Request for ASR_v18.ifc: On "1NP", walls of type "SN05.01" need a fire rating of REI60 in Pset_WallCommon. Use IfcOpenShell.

First a look at what the model holds.

```python
import ifcopenshell
import ifcopenshell.util.element

model = ifcopenshell.open("ASR_v18.ifc")
print(model.schema)
storey = next(s for s in model.by_type("IfcBuildingStorey") if s.Name == "1NP")
walls = [e for e in ifcopenshell.util.element.get_decomposition(storey) if e.is_a("IfcWall")]
seen = {}
for e in walls:
    element_type = ifcopenshell.util.element.get_type(e)
    key = (element_type.Name if element_type != e and element_type else None, ifcopenshell.util.element.get_pset(e, "Pset_WallCommon", "FireRating"))
    seen[key] = seen.get(key, 0) + 1
for (name, value), count in sorted(seen.items(), key=str):
    print(count, "x", name, "|", value)
```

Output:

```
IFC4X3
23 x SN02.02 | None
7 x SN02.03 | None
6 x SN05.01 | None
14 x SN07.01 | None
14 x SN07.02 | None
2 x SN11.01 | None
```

```python
import ifcopenshell
import ifcopenshell.api.pset
import ifcopenshell.util.element

model = ifcopenshell.open("ASR_v18.ifc")

storey = next(s for s in model.by_type("IfcBuildingStorey") if s.Name == "1NP")
walls = [e for e in ifcopenshell.util.element.get_decomposition(storey) if e.is_a("IfcWall")]

count = 0
for e in walls:
    element_type = ifcopenshell.util.element.get_type(e)
    if element_type in (None, e) or element_type.Name != "SN05.01":
        continue
    # add_pset returns the element's existing set when there is one.
    pset = ifcopenshell.api.pset.add_pset(model, product=e, name="Pset_WallCommon")
    ifcopenshell.api.pset.edit_pset(model, pset=pset, properties={"FireRating": "REI60"})
    count += 1

print(count, "walls updated")

model.write("ASR_v18-out.ifc")
```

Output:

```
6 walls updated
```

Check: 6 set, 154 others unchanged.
